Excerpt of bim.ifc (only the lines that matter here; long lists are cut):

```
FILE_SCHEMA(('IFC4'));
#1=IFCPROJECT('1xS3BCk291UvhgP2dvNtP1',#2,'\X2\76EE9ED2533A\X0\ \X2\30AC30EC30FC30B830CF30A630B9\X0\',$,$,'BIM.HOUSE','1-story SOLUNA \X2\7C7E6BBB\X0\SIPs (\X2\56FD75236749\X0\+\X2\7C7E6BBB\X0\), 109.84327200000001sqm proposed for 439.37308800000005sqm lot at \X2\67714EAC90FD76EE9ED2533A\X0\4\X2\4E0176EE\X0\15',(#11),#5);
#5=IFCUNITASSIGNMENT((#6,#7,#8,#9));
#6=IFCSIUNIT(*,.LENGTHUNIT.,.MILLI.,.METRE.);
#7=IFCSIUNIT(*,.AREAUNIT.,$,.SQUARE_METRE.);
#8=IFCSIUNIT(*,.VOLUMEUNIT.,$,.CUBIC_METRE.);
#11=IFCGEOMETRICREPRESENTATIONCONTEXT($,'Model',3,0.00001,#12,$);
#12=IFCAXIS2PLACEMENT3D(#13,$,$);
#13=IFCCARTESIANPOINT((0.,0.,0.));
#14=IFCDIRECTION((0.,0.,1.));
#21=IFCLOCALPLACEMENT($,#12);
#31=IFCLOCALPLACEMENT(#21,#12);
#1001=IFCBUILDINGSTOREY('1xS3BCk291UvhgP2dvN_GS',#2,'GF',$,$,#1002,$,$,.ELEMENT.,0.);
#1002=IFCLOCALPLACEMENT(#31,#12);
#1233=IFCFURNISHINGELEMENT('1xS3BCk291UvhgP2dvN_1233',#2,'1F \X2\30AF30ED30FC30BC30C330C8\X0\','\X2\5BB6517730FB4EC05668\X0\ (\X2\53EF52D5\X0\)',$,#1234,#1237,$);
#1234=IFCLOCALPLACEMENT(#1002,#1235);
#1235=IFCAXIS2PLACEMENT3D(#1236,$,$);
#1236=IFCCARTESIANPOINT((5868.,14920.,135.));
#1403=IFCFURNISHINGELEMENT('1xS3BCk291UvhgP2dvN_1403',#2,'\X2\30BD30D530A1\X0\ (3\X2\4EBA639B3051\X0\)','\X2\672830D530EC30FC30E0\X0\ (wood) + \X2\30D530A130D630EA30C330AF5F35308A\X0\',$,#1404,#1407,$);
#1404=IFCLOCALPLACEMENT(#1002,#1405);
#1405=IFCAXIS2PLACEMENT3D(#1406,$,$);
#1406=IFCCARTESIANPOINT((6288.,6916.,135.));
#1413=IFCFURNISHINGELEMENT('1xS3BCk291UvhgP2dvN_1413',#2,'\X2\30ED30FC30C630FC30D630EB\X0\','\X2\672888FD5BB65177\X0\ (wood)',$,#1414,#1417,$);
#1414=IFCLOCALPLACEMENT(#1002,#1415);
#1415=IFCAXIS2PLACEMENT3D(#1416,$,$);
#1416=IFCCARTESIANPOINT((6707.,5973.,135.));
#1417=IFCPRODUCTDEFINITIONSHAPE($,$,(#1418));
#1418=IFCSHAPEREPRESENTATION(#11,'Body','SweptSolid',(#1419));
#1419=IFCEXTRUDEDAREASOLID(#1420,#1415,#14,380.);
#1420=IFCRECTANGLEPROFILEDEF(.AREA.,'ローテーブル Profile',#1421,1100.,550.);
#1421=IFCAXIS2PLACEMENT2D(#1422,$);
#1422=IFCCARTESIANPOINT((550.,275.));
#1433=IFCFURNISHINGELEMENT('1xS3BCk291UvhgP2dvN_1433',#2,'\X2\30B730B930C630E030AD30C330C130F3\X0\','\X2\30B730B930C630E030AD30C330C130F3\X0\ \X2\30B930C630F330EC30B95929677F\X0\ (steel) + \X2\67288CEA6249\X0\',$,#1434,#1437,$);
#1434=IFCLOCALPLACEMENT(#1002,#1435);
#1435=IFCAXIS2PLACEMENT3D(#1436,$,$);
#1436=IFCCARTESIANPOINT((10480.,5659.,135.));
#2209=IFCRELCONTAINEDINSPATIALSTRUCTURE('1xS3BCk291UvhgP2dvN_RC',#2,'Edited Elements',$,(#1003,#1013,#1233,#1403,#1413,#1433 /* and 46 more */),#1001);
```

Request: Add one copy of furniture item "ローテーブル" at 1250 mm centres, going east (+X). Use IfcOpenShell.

```python
import numpy as np
import ifcopenshell
import ifcopenshell.api.geometry
import ifcopenshell.api.root
import ifcopenshell.util.element
import ifcopenshell.util.placement
import ifcopenshell.util.unit

model = ifcopenshell.open("bim.ifc")
unit_scale = ifcopenshell.util.unit.calculate_unit_scale(model)


def reuse_history(source, copy):
    """copy_class also copies each property set's owner history, people and application; keep the originals."""
    for rel in copy.IsDefinedBy:
        if rel.is_a("IfcRelDefinesByProperties") and (history := rel.RelatingPropertyDefinition.OwnerHistory):
            rel.RelatingPropertyDefinition.OwnerHistory = source.OwnerHistory
            ifcopenshell.util.element.remove_deep2(model, history)


source = model.by_guid("1xS3BCk291UvhgP2dvN_1413")
base = ifcopenshell.util.placement.get_local_placement(source.ObjectPlacement)
step = np.array([1.0, 0.0, 0.0]) * 1.25 / unit_scale

for i in range(1, 2):
    copy = ifcopenshell.api.root.copy_class(model, product=source)
    copy.Representation = ifcopenshell.util.element.copy_deep(
        model, source.Representation, exclude=["IfcGeometricRepresentationContext", "IfcRepresentationMap"]
    )
    reuse_history(source, copy)
    matrix = base.copy()
    matrix[:3, 3] += i * step
    print("added at", matrix[:3, 3].round(3) + 0.0)
    ifcopenshell.api.geometry.edit_object_placement(model, product=copy, matrix=matrix, is_si=False)

model.write("bim_edited.ifc")
```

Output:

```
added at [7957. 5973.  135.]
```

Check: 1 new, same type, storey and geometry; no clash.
